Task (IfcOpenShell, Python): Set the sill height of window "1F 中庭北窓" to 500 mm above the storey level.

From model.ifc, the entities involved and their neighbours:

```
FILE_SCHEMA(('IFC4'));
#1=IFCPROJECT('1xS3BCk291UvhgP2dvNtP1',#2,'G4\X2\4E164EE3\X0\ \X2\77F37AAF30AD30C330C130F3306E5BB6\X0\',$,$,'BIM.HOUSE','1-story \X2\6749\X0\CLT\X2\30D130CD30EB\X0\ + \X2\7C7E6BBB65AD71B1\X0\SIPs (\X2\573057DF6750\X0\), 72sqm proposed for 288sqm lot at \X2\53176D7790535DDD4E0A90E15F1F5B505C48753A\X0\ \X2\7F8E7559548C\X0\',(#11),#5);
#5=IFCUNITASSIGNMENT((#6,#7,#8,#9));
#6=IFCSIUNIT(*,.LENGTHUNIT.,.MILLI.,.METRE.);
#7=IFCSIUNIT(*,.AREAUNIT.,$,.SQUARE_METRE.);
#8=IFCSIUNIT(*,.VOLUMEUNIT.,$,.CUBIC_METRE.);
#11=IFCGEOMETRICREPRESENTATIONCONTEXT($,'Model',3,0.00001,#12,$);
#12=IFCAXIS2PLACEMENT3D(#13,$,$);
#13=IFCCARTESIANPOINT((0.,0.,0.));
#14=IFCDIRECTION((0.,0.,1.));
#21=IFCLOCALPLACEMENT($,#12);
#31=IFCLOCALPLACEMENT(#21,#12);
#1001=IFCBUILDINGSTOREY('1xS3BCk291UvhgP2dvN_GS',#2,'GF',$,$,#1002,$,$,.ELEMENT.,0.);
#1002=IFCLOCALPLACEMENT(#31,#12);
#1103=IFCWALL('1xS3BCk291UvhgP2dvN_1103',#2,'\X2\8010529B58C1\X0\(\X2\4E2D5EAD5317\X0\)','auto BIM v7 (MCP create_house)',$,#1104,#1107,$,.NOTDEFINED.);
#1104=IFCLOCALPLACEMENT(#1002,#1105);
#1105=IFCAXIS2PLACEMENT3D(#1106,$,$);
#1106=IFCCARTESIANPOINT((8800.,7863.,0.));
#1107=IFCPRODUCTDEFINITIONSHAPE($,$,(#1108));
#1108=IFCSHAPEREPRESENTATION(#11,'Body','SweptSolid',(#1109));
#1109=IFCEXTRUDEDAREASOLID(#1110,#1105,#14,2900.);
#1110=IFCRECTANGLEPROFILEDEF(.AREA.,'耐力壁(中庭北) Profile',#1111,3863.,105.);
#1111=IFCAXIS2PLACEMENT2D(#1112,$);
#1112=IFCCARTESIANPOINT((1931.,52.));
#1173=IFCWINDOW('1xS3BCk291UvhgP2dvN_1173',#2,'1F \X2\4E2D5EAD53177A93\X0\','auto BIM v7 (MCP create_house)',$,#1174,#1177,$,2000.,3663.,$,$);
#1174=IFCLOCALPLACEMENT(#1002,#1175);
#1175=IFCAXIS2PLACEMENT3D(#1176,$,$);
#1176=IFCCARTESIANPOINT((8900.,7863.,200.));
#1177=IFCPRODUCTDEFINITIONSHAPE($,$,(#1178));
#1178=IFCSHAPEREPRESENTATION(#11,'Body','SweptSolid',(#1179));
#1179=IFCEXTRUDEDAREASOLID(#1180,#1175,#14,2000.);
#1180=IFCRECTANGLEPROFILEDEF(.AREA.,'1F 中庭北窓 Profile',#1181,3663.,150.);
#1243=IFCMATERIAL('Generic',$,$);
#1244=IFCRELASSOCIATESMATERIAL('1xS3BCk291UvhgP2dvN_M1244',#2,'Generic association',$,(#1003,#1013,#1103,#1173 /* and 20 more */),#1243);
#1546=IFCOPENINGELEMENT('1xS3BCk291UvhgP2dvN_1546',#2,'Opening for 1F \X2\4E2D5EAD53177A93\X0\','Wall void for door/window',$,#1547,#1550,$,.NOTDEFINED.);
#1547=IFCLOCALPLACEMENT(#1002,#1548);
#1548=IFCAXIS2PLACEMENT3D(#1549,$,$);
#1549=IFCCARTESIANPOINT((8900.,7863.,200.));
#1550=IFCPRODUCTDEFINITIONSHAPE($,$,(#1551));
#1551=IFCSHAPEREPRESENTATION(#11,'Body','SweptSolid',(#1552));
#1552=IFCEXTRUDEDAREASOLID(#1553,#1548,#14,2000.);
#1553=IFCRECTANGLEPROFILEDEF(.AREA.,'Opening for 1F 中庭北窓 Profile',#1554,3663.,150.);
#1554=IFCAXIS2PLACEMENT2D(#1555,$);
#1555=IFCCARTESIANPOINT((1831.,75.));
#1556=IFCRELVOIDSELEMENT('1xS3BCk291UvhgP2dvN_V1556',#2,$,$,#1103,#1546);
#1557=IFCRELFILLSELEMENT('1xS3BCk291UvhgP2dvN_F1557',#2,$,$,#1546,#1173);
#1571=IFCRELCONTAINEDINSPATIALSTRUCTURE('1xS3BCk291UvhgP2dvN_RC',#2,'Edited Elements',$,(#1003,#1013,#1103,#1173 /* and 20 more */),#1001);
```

```python
import numpy as np
import ifcopenshell
import ifcopenshell.api.geometry
import ifcopenshell.geom
import ifcopenshell.util.element
import ifcopenshell.util.placement
import ifcopenshell.util.shape
import ifcopenshell.util.unit

model = ifcopenshell.open("model.ifc")
unit_scale = ifcopenshell.util.unit.calculate_unit_scale(model)

window = model.by_guid("1xS3BCk291UvhgP2dvN_1173")
opening = window.FillsVoids[0].RelatingOpeningElement
storey = ifcopenshell.util.element.get_container(window, ifc_class="IfcBuildingStorey")
level = ifcopenshell.util.placement.get_local_placement(storey.ObjectPlacement)[2, 3]

# The opening's origin need not be at the sill, so measure its lowest point.
shape = ifcopenshell.geom.create_shape(ifcopenshell.geom.settings(), opening)
bottom = ifcopenshell.util.shape.get_shape_bottom_elevation(shape, shape.geometry) / unit_scale
dz = level + 0.5 / unit_scale - bottom

shift = np.array([0.0, 0.0, dz])
# The window is not placed relative to its opening, so move both.
for product in (opening, window):
    matrix = ifcopenshell.util.placement.get_local_placement(product.ObjectPlacement)
    matrix[:3, 3] += shift
    ifcopenshell.api.geometry.edit_object_placement(model, product=product, matrix=matrix, is_si=False)

print(f"moved by {dz * unit_scale:+.3f} m")

model.write("model_edited.ifc")
```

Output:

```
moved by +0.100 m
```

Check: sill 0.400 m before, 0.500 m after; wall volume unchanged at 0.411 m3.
